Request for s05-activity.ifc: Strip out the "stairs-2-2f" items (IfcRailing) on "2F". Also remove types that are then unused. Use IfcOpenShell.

First a look at what the model holds.

```python
import ifcopenshell
import ifcopenshell.util.element

model = ifcopenshell.open("s05-activity.ifc")
print(model.schema)
storey = next(s for s in model.by_type("IfcBuildingStorey") if s.Name == "2F")
railings = [e for e in ifcopenshell.util.element.get_decomposition(storey) if e.is_a("IfcRailing")]
seen = {}
for e in railings:
    element_type = ifcopenshell.util.element.get_type(e)
    name = element_type.Name if element_type not in (None, e) else None
    seen[name] = seen.get(name, 0) + 1
for name, count in sorted(seen.items(), key=str):
    print(count, "x", name)
```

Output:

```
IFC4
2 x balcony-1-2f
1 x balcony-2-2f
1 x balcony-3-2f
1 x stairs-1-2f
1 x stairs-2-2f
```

```python
import ifcopenshell
import ifcopenshell.api.root
import ifcopenshell.util.element

model = ifcopenshell.open("s05-activity.ifc")

storey = next(s for s in model.by_type("IfcBuildingStorey") if s.Name == "2F")
railings = [e for e in ifcopenshell.util.element.get_decomposition(storey) if e.is_a("IfcRailing")]
targets = [e for e in railings if (t := ifcopenshell.util.element.get_type(e)) not in (None, e) and t.Name == "stairs-2-2f"]
types = {ifcopenshell.util.element.get_type(e) for e in targets} - {None, *targets}

for e in targets:
    ifcopenshell.api.root.remove_product(model, product=e)
print(len(targets), "removed")

unused = [t for t in types if not ifcopenshell.util.element.get_types(t)]
for t in unused:
    ifcopenshell.api.root.remove_product(model, product=t)
print(len(unused), "unused types removed")

model.write("s05-activity-out.ifc")
```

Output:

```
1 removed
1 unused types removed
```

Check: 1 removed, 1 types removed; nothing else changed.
